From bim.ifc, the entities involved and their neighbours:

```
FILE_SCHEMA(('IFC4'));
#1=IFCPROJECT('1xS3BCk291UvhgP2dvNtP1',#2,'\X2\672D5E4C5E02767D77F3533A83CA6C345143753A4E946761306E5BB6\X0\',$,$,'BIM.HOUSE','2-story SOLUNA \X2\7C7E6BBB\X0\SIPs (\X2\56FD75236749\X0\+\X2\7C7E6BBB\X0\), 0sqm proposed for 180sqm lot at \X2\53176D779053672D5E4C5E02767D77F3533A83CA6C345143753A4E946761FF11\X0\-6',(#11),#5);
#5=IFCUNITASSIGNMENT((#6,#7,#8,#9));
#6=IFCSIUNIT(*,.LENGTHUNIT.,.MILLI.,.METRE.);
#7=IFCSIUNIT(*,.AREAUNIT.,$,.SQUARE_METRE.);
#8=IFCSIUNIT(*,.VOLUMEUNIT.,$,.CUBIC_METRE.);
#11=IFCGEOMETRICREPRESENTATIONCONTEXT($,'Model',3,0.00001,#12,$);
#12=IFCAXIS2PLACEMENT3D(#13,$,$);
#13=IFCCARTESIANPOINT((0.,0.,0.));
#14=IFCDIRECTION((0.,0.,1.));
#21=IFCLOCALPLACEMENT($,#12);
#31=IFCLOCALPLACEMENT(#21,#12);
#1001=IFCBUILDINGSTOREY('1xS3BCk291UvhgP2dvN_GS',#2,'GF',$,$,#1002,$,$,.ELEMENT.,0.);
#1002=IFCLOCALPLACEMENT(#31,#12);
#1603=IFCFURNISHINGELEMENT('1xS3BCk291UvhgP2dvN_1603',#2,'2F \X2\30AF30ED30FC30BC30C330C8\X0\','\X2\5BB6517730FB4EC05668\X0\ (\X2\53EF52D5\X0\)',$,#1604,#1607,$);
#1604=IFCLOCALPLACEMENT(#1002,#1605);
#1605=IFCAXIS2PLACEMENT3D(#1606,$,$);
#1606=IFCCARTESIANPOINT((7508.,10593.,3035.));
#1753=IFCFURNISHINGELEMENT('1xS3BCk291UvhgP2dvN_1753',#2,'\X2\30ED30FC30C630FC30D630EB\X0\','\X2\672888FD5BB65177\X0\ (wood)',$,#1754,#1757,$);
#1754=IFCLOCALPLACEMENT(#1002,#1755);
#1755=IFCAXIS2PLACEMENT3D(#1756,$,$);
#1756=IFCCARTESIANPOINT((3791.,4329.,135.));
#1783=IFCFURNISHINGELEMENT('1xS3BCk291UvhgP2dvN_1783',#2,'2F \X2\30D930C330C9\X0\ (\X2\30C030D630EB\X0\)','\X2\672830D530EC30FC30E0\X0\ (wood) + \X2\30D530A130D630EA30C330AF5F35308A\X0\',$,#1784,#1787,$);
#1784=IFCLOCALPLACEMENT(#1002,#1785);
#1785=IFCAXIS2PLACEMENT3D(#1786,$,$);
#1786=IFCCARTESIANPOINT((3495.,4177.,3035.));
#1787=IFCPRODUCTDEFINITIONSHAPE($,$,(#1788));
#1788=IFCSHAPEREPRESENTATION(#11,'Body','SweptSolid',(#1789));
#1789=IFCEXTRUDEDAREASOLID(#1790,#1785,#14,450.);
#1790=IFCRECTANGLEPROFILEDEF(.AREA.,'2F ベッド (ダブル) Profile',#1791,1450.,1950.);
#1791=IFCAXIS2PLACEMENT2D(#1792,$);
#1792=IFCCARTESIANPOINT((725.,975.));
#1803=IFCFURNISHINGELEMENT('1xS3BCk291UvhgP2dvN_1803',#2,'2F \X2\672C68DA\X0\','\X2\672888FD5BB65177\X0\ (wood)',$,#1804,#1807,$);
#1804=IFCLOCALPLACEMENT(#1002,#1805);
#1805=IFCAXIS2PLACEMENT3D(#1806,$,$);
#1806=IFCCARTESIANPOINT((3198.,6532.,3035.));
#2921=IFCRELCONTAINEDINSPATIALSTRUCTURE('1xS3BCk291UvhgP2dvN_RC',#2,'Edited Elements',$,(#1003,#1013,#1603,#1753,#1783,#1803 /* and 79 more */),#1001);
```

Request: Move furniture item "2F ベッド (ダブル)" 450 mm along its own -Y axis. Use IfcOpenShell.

```python
import ifcopenshell
import ifcopenshell.api.geometry
import ifcopenshell.util.placement
import ifcopenshell.util.unit

model = ifcopenshell.open("bim.ifc")
unit_scale = ifcopenshell.util.unit.calculate_unit_scale(model)

item = model.by_id(1783)
matrix = ifcopenshell.util.placement.get_local_placement(item.ObjectPlacement)
matrix[:3, 3] -= matrix[:3, 1] * 0.45 / unit_scale
ifcopenshell.api.geometry.edit_object_placement(model, product=item, matrix=matrix, is_si=False)

print(ifcopenshell.util.placement.get_local_placement(item.ObjectPlacement).round(3) + 0.0)

model.write("bim_v2.ifc")
```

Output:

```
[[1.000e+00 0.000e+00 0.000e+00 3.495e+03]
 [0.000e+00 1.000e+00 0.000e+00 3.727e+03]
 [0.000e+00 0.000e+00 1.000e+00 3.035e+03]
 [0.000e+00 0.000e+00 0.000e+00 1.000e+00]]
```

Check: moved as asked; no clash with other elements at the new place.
